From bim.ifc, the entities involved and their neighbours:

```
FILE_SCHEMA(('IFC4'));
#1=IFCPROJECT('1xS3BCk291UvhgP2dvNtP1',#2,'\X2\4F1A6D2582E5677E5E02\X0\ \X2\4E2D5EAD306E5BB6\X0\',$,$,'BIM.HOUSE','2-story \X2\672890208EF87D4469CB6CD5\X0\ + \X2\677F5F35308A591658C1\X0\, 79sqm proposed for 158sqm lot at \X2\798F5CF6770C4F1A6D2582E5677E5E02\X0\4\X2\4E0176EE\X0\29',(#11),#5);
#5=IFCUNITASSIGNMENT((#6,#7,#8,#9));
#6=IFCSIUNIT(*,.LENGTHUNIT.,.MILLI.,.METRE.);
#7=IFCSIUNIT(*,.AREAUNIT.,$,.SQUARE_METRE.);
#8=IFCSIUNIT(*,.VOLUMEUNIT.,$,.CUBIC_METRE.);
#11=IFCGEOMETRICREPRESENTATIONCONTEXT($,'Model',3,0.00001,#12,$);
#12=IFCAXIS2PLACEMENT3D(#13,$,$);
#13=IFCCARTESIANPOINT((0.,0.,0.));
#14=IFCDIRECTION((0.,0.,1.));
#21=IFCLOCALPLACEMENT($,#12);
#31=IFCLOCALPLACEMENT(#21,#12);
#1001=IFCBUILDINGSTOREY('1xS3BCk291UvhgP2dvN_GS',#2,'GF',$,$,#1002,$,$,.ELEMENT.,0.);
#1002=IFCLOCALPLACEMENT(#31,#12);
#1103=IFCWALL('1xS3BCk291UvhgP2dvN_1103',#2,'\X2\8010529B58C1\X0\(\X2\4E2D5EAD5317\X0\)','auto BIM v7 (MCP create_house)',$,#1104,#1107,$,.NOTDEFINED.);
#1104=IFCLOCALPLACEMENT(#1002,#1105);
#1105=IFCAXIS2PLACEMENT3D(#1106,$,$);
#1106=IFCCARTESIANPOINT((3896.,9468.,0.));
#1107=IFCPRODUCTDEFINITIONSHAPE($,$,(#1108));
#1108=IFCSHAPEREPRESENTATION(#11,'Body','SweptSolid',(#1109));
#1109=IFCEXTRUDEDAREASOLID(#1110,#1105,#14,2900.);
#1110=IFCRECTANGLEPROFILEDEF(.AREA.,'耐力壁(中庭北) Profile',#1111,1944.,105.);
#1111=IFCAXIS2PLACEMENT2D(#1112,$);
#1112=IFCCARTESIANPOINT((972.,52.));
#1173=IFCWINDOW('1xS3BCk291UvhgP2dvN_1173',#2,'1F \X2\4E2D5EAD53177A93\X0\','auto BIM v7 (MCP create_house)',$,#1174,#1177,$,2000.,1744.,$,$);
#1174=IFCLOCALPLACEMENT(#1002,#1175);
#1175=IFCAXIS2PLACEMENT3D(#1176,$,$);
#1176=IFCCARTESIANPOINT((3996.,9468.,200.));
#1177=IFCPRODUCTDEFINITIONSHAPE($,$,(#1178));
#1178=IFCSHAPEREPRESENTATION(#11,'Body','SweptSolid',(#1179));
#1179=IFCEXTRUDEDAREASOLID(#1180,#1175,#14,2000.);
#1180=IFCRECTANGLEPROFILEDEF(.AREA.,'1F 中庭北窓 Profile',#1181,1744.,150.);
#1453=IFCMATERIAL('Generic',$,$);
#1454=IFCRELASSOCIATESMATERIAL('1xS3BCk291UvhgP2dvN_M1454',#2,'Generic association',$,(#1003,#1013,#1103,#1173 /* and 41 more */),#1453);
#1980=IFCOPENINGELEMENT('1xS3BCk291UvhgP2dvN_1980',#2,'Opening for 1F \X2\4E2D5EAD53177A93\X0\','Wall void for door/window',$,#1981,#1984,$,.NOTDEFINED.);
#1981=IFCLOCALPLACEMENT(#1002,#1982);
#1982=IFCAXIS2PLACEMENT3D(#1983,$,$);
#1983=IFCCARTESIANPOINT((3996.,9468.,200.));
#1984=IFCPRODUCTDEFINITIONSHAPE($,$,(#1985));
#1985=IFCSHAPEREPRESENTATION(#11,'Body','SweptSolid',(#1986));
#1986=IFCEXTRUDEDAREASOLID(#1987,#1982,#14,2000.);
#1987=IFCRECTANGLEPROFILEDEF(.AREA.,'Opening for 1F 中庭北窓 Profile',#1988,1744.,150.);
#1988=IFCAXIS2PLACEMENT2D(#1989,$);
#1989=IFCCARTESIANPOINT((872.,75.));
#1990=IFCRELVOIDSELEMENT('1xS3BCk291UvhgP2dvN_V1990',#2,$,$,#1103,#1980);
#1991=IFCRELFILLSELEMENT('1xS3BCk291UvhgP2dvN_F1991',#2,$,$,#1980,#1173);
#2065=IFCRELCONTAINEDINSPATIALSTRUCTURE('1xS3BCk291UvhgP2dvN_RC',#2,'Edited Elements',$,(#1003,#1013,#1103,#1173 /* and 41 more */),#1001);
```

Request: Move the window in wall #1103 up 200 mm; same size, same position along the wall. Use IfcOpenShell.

```python
import numpy as np
import ifcopenshell
import ifcopenshell.api.geometry
import ifcopenshell.util.placement
import ifcopenshell.util.unit

model = ifcopenshell.open("bim.ifc")
unit_scale = ifcopenshell.util.unit.calculate_unit_scale(model)

window = model.by_guid("1xS3BCk291UvhgP2dvN_1173")
opening = window.FillsVoids[0].RelatingOpeningElement
dz = 0.2 / unit_scale

shift = np.array([0.0, 0.0, dz])
# The window is not placed relative to its opening, so move both.
for product in (opening, window):
    matrix = ifcopenshell.util.placement.get_local_placement(product.ObjectPlacement)
    matrix[:3, 3] += shift
    ifcopenshell.api.geometry.edit_object_placement(model, product=product, matrix=matrix, is_si=False)

print(f"moved by {dz * unit_scale:+.3f} m")

model.write("bim_edited.ifc")
```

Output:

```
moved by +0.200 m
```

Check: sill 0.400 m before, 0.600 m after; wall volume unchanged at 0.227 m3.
